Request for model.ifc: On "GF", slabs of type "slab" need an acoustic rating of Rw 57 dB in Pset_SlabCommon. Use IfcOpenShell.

First a look at what the model holds.

```python
import ifcopenshell
import ifcopenshell.util.element

model = ifcopenshell.open("model.ifc")
print(model.schema)
storey = next(s for s in model.by_type("IfcBuildingStorey") if s.Name == "GF")
slabs = [e for e in ifcopenshell.util.element.get_decomposition(storey) if e.is_a("IfcSlab")]
seen = {}
for e in slabs:
    element_type = ifcopenshell.util.element.get_type(e)
    key = (element_type.Name if element_type != e and element_type else None, ifcopenshell.util.element.get_pset(e, "Pset_SlabCommon", "AcousticRating"))
    seen[key] = seen.get(key, 0) + 1
for (name, value), count in sorted(seen.items(), key=str):
    print(count, "x", name, "|", value)
```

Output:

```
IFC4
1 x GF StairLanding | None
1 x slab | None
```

```python
import ifcopenshell
import ifcopenshell.api.pset
import ifcopenshell.util.element

model = ifcopenshell.open("model.ifc")

storey = next(s for s in model.by_type("IfcBuildingStorey") if s.Name == "GF")
slabs = [e for e in ifcopenshell.util.element.get_decomposition(storey) if e.is_a("IfcSlab")]

count = 0
for e in slabs:
    element_type = ifcopenshell.util.element.get_type(e)
    if element_type in (None, e) or element_type.Name != "slab":
        continue
    # add_pset returns the element's existing set when there is one.
    pset = ifcopenshell.api.pset.add_pset(model, product=e, name="Pset_SlabCommon")
    ifcopenshell.api.pset.edit_pset(model, pset=pset, properties={"AcousticRating": "Rw 57 dB"})
    count += 1

print(count, "slabs updated")

model.write("model-out.ifc")
```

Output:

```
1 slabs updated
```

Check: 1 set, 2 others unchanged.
